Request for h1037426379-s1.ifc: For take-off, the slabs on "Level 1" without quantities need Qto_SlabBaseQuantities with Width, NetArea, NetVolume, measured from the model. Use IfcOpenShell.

First a look at what the model holds.

```python
import ifcopenshell
import ifcopenshell.util.element
import ifcopenshell.util.unit

model = ifcopenshell.open("h1037426379-s1.ifc")
print(model.schema)
for unit_type in ("LENGTHUNIT", "AREAUNIT", "VOLUMEUNIT"):
    print(unit_type, ifcopenshell.util.unit.calculate_unit_scale(model, unit_type))
storey = next(s for s in model.by_type("IfcBuildingStorey") if s.Name == "Level 1")
slabs = [e for e in ifcopenshell.util.element.get_decomposition(storey) if e.is_a("IfcSlab")]
for e in sorted(slabs, key=lambda e: e.id()):
    print(e.id(), e.is_a(), e.Name, list(ifcopenshell.util.element.get_psets(e, qtos_only=True)), sep=" | ")
```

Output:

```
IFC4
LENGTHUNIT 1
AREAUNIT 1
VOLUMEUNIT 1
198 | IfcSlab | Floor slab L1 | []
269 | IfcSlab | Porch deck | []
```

```python
import ifcopenshell
import ifcopenshell.api.pset
import ifcopenshell.geom
import ifcopenshell.util.element
import ifcopenshell.util.shape
import ifcopenshell.util.unit

model = ifcopenshell.open("h1037426379-s1.ifc")
unit_scale = ifcopenshell.util.unit.calculate_unit_scale(model)
area_scale = ifcopenshell.util.unit.calculate_unit_scale(model, "AREAUNIT")
volume_scale = ifcopenshell.util.unit.calculate_unit_scale(model, "VOLUMEUNIT")
settings = ifcopenshell.geom.settings()

storey = next(s for s in model.by_type("IfcBuildingStorey") if s.Name == "Level 1")
slabs = [e for e in ifcopenshell.util.element.get_decomposition(storey) if e.is_a("IfcSlab")]

for e in sorted(slabs, key=lambda e: e.id()):
    if ifcopenshell.util.element.get_psets(e, qtos_only=True, should_inherit=False):
        continue
    # Geometry comes back in metres, in the element's own axes.
    shape = ifcopenshell.geom.create_shape(settings, e)
    values = {
        "Width": ifcopenshell.util.shape.get_z(shape.geometry) / unit_scale,
        "NetArea": ifcopenshell.util.shape.get_footprint_area(shape.geometry) / area_scale,
        "NetVolume": ifcopenshell.util.shape.get_volume(shape.geometry) / volume_scale,
    }
    qto = ifcopenshell.api.pset.add_qto(model, product=e, name="Qto_SlabBaseQuantities")
    ifcopenshell.api.pset.edit_qto(model, qto=qto, properties=values)
    print(e.id(), {k: round(v, 3) for k, v in values.items()})

model.write("h1037426379-s1_rev.ifc")
```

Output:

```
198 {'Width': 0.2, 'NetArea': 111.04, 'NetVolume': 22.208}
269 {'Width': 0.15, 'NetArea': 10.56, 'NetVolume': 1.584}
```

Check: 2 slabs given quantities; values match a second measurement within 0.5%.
